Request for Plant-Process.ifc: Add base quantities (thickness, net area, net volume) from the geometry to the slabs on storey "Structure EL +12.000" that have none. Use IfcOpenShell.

First a look at what the model holds.

```python
import ifcopenshell
import ifcopenshell.util.element
import ifcopenshell.util.unit

model = ifcopenshell.open("Plant-Process.ifc")
print(model.schema)
for unit_type in ("LENGTHUNIT", "AREAUNIT", "VOLUMEUNIT"):
    print(unit_type, ifcopenshell.util.unit.calculate_unit_scale(model, unit_type))
storey = next(s for s in model.by_type("IfcBuildingStorey") if s.Name == "Structure EL +12.000")
slabs = [e for e in ifcopenshell.util.element.get_decomposition(storey) if e.is_a("IfcSlab")]
for e in sorted(slabs, key=lambda e: e.id()):
    print(e.id(), e.is_a(), e.Name, list(ifcopenshell.util.element.get_psets(e, qtos_only=True)), sep=" | ")
```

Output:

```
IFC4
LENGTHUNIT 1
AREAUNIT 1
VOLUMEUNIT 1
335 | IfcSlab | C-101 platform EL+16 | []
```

```python
import ifcopenshell
import ifcopenshell.api.pset
import ifcopenshell.geom
import ifcopenshell.util.element
import ifcopenshell.util.shape
import ifcopenshell.util.unit

model = ifcopenshell.open("Plant-Process.ifc")
unit_scale = ifcopenshell.util.unit.calculate_unit_scale(model)
area_scale = ifcopenshell.util.unit.calculate_unit_scale(model, "AREAUNIT")
volume_scale = ifcopenshell.util.unit.calculate_unit_scale(model, "VOLUMEUNIT")
settings = ifcopenshell.geom.settings()

storey = next(s for s in model.by_type("IfcBuildingStorey") if s.Name == "Structure EL +12.000")
slabs = [e for e in ifcopenshell.util.element.get_decomposition(storey) if e.is_a("IfcSlab")]

for e in sorted(slabs, key=lambda e: e.id()):
    if ifcopenshell.util.element.get_psets(e, qtos_only=True, should_inherit=False):
        continue
    # Geometry comes back in metres, in the element's own axes.
    shape = ifcopenshell.geom.create_shape(settings, e)
    values = {
        "Width": ifcopenshell.util.shape.get_z(shape.geometry) / unit_scale,
        "NetArea": ifcopenshell.util.shape.get_footprint_area(shape.geometry) / area_scale,
        "NetVolume": ifcopenshell.util.shape.get_volume(shape.geometry) / volume_scale,
    }
    qto = ifcopenshell.api.pset.add_qto(model, product=e, name="Qto_SlabBaseQuantities")
    ifcopenshell.api.pset.edit_qto(model, qto=qto, properties=values)
    print(e.id(), {k: round(v, 3) for k, v in values.items()})

model.write("Plant-Process-out.ifc")
```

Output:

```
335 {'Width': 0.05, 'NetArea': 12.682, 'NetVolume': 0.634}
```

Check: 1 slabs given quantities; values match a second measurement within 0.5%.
